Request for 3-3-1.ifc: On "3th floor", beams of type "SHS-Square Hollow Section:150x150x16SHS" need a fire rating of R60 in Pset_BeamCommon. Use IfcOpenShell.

First a look at what the model holds.

```python
import ifcopenshell
import ifcopenshell.util.element

model = ifcopenshell.open("3-3-1.ifc")
print(model.schema)
storey = next(s for s in model.by_type("IfcBuildingStorey") if s.Name == "3th floor")
beams = [e for e in ifcopenshell.util.element.get_decomposition(storey) if e.is_a("IfcBeam")]
seen = {}
for e in beams:
    element_type = ifcopenshell.util.element.get_type(e)
    key = (element_type.Name if element_type != e and element_type else None, ifcopenshell.util.element.get_pset(e, "Pset_BeamCommon", "FireRating"))
    seen[key] = seen.get(key, 0) + 1
for (name, value), count in sorted(seen.items(), key=str):
    print(count, "x", name, "|", value)
```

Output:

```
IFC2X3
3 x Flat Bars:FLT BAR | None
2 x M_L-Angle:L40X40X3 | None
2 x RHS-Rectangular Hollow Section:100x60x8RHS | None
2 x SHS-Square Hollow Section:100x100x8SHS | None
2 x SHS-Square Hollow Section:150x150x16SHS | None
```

```python
import ifcopenshell
import ifcopenshell.api.pset
import ifcopenshell.util.element

model = ifcopenshell.open("3-3-1.ifc")

storey = next(s for s in model.by_type("IfcBuildingStorey") if s.Name == "3th floor")
beams = [e for e in ifcopenshell.util.element.get_decomposition(storey) if e.is_a("IfcBeam")]

count = 0
for e in beams:
    element_type = ifcopenshell.util.element.get_type(e)
    if element_type in (None, e) or element_type.Name != "SHS-Square Hollow Section:150x150x16SHS":
        continue
    # add_pset returns the element's existing set when there is one.
    pset = ifcopenshell.api.pset.add_pset(model, product=e, name="Pset_BeamCommon")
    ifcopenshell.api.pset.edit_pset(model, pset=pset, properties={"FireRating": "R60"})
    count += 1

print(count, "beams updated")

model.write("3-3-1_v2.ifc")
```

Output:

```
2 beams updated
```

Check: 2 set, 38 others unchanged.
